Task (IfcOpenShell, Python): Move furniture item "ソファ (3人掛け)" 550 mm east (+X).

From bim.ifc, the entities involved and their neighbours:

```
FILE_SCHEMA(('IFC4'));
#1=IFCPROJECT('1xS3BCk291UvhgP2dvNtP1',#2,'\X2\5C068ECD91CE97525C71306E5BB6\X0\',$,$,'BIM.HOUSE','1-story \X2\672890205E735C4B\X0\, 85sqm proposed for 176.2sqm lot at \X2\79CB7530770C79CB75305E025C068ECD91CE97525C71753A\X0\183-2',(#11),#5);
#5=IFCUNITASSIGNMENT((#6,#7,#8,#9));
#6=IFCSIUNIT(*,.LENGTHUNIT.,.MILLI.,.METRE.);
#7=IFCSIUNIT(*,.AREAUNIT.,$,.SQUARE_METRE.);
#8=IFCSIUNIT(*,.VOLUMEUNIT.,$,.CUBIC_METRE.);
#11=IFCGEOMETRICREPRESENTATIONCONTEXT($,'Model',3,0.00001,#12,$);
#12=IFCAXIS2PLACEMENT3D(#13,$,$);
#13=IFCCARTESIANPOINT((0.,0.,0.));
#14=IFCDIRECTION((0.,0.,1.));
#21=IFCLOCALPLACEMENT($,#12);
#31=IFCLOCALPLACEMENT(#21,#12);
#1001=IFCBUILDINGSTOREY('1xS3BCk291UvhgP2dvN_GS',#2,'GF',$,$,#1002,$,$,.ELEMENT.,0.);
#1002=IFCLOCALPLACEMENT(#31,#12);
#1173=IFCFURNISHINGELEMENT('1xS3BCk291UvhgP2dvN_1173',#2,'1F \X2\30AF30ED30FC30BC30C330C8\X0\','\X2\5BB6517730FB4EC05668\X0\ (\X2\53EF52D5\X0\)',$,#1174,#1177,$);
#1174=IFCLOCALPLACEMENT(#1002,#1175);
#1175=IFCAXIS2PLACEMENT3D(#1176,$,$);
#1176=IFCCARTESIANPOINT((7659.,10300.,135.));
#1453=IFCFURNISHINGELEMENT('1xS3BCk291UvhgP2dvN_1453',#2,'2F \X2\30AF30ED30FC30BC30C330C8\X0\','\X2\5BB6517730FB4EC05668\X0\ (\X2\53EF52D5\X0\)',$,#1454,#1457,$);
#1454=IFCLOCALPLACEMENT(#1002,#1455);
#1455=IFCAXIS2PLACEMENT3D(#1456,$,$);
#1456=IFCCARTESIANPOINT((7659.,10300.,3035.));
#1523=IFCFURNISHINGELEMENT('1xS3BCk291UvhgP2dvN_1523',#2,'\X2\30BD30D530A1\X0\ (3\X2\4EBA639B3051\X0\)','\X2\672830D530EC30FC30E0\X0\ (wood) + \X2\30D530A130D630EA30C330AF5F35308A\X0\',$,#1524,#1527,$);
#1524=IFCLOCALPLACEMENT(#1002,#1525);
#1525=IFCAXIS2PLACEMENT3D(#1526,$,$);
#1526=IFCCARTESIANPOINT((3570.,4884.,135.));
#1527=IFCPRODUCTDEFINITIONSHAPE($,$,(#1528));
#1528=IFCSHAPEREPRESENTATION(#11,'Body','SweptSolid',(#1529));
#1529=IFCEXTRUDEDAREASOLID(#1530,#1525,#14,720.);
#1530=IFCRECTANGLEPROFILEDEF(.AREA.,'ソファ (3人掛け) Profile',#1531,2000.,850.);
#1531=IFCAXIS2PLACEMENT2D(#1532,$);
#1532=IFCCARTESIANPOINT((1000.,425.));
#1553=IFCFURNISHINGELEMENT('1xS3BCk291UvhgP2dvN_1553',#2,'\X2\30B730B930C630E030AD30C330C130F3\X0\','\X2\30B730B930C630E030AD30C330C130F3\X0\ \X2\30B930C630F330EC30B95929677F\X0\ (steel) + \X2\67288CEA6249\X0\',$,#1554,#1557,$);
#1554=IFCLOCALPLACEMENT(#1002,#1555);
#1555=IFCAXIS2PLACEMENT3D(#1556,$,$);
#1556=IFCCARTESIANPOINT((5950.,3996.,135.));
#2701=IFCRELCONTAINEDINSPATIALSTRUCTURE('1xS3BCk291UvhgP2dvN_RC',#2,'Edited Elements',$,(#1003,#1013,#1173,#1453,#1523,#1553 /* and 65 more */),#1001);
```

```python
import ifcopenshell
import ifcopenshell.api.geometry
import ifcopenshell.util.placement
import ifcopenshell.util.unit

model = ifcopenshell.open("bim.ifc")
unit_scale = ifcopenshell.util.unit.calculate_unit_scale(model)

item = model.by_id(1523)
matrix = ifcopenshell.util.placement.get_local_placement(item.ObjectPlacement)
matrix[0, 3] += 0.55 / unit_scale
ifcopenshell.api.geometry.edit_object_placement(model, product=item, matrix=matrix, is_si=False)

print(ifcopenshell.util.placement.get_local_placement(item.ObjectPlacement).round(3) + 0.0)

model.write("bim_edited.ifc")
```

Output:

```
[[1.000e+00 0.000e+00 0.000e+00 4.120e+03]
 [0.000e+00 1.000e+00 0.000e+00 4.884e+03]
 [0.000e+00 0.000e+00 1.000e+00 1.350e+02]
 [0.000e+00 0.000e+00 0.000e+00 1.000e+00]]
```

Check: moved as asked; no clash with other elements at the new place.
